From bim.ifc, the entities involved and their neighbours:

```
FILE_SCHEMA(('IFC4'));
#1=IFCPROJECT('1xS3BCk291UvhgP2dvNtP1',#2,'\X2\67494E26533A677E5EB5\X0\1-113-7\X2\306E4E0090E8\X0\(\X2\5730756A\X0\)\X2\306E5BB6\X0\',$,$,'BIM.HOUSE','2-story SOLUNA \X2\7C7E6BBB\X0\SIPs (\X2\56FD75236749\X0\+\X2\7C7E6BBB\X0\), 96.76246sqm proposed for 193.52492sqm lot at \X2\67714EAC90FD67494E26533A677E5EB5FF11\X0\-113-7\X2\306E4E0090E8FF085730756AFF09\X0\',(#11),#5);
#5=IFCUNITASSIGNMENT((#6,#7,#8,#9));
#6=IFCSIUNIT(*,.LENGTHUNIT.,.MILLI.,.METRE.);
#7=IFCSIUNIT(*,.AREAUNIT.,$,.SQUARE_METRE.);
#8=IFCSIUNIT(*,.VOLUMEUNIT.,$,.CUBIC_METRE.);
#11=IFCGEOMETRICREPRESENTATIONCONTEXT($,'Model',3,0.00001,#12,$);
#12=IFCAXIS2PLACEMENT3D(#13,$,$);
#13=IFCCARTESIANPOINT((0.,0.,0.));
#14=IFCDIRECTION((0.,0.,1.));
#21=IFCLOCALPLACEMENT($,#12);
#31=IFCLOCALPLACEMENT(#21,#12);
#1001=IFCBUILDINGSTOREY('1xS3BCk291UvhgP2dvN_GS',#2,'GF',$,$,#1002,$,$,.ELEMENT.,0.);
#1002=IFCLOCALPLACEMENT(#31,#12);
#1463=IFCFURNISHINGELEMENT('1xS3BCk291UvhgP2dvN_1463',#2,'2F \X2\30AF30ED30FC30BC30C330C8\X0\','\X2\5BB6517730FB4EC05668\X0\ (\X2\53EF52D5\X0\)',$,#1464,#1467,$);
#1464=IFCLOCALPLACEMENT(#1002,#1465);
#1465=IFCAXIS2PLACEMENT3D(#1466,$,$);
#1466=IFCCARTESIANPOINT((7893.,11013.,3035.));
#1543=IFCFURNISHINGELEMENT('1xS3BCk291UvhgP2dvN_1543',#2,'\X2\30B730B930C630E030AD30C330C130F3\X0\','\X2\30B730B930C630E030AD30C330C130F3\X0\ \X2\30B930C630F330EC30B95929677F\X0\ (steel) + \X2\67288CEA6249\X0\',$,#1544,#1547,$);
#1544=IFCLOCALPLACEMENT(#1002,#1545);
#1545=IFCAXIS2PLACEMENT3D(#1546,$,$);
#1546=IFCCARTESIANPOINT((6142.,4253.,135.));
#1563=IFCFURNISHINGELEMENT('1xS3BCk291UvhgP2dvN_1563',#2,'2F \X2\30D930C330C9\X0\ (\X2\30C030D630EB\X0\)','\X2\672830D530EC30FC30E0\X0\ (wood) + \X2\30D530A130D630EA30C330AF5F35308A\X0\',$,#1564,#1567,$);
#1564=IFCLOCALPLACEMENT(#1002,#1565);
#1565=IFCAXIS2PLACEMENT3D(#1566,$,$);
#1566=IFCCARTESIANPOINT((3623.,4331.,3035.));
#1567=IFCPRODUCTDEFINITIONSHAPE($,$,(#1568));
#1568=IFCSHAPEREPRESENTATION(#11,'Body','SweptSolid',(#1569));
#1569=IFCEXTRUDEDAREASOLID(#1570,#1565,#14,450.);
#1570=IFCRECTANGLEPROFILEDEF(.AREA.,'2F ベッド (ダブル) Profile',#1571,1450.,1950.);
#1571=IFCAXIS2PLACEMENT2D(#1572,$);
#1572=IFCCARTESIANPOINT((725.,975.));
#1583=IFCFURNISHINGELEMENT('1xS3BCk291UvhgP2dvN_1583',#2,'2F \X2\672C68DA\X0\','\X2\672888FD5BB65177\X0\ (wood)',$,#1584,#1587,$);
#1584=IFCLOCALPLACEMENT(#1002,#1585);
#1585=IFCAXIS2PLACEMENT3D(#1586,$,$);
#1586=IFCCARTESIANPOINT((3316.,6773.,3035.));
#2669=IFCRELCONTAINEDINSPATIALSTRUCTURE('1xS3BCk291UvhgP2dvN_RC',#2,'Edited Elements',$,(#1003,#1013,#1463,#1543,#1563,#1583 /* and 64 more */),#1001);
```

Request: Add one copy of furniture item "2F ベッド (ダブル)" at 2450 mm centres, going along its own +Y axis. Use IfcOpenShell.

```python
import ifcopenshell
import ifcopenshell.api.geometry
import ifcopenshell.api.root
import ifcopenshell.util.element
import ifcopenshell.util.placement
import ifcopenshell.util.unit

model = ifcopenshell.open("bim.ifc")
unit_scale = ifcopenshell.util.unit.calculate_unit_scale(model)


def reuse_history(source, copy):
    """copy_class also copies each property set's owner history, people and application; keep the originals."""
    for rel in copy.IsDefinedBy:
        if rel.is_a("IfcRelDefinesByProperties") and (history := rel.RelatingPropertyDefinition.OwnerHistory):
            rel.RelatingPropertyDefinition.OwnerHistory = source.OwnerHistory
            ifcopenshell.util.element.remove_deep2(model, history)


source = model.by_guid("1xS3BCk291UvhgP2dvN_1563")
base = ifcopenshell.util.placement.get_local_placement(source.ObjectPlacement)
step = base[:3, 1] * 2.45 / unit_scale

for i in range(1, 2):
    copy = ifcopenshell.api.root.copy_class(model, product=source)
    copy.Representation = ifcopenshell.util.element.copy_deep(
        model, source.Representation, exclude=["IfcGeometricRepresentationContext", "IfcRepresentationMap"]
    )
    reuse_history(source, copy)
    matrix = base.copy()
    matrix[:3, 3] += i * step
    print("added at", matrix[:3, 3].round(3) + 0.0)
    ifcopenshell.api.geometry.edit_object_placement(model, product=copy, matrix=matrix, is_si=False)

model.write("bim-out.ifc")
```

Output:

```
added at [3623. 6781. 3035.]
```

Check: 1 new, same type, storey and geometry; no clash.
